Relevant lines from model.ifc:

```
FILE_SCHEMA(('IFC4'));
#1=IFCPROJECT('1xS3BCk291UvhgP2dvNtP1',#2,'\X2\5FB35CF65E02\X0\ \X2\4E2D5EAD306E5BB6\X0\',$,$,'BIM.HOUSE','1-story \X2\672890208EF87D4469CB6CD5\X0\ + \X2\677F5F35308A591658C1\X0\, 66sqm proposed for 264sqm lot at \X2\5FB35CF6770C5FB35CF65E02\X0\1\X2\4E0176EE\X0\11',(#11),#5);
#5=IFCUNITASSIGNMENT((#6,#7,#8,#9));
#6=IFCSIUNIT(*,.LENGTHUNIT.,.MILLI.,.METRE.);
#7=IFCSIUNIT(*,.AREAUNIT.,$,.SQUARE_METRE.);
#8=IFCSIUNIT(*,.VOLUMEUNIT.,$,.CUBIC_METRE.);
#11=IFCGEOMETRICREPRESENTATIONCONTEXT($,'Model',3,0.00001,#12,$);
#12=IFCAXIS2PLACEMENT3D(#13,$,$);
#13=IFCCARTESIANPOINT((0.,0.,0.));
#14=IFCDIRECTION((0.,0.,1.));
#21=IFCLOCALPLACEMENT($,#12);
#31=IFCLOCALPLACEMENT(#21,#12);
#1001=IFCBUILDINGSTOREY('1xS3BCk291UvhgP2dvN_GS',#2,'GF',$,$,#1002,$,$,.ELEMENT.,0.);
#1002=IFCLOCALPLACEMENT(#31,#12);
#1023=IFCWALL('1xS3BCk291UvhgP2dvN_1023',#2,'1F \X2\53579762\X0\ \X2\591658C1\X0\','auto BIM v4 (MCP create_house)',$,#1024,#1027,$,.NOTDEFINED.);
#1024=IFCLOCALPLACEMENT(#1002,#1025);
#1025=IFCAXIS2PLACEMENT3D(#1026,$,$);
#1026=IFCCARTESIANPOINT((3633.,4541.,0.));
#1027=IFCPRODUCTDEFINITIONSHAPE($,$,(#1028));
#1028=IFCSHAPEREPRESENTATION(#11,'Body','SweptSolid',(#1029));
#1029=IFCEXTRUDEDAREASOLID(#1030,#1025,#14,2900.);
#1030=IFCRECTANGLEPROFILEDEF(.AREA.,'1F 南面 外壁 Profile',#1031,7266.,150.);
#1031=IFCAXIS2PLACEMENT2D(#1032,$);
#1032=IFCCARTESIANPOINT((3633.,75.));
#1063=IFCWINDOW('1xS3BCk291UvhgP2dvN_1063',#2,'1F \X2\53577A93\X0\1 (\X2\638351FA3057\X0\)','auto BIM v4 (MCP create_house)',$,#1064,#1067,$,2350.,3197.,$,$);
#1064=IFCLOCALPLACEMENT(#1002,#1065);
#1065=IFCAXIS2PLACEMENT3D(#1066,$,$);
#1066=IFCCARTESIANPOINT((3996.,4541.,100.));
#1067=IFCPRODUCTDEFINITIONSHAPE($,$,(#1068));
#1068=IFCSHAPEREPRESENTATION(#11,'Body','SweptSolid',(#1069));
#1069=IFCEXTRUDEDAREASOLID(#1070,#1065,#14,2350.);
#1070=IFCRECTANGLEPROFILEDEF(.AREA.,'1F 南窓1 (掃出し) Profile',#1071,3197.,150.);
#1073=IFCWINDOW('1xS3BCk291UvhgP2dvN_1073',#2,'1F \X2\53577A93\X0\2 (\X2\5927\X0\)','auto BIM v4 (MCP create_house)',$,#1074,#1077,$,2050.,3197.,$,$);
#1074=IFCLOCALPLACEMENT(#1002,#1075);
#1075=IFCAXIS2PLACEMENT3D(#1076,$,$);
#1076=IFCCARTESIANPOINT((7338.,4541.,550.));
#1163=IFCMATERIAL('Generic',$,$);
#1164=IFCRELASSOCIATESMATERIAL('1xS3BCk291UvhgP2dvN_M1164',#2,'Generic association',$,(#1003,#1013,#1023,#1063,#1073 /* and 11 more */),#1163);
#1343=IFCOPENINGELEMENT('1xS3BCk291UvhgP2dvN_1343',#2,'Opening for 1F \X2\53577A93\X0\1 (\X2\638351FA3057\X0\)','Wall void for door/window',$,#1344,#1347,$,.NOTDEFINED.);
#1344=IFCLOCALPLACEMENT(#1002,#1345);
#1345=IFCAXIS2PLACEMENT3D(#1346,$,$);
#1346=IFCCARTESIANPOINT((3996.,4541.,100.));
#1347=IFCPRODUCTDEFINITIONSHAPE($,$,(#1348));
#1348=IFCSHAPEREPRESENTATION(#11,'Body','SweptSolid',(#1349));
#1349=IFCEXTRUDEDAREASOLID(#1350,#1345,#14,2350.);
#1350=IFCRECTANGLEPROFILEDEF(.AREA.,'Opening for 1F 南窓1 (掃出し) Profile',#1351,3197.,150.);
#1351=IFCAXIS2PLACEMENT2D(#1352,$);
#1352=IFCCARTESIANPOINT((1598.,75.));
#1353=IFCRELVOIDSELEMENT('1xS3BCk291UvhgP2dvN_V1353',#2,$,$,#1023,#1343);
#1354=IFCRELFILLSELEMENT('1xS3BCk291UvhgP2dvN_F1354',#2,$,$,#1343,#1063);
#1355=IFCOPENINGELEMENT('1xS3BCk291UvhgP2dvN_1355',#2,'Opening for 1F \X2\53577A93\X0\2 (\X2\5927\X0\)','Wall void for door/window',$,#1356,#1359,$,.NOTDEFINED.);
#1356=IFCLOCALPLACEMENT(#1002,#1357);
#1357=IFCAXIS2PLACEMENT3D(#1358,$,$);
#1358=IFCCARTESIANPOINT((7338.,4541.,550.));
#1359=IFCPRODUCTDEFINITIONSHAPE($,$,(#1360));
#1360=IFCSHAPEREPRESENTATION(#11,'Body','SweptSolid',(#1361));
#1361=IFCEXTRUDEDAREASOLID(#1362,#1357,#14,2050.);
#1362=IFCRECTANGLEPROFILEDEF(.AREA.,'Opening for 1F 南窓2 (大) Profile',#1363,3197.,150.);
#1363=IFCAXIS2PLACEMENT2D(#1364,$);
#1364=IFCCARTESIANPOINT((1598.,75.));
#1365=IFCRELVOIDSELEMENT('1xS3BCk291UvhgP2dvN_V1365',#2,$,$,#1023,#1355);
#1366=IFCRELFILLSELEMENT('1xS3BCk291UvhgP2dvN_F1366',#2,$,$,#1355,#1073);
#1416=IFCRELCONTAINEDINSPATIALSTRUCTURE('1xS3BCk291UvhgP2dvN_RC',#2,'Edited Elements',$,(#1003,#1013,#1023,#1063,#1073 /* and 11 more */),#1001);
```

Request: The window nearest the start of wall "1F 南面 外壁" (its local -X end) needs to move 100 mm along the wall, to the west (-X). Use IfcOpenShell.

```python
import ifcopenshell
import ifcopenshell.api.geometry
import ifcopenshell.util.placement

model = ifcopenshell.open("model.ifc")

window = model.by_guid("1xS3BCk291UvhgP2dvN_1063")
opening = window.FillsVoids[0].RelatingOpeningElement
wall = opening.VoidsElements[0].RelatingBuildingElement

wall_matrix = ifcopenshell.util.placement.get_local_placement(wall.ObjectPlacement)
shift = wall_matrix[:3, 0] * -100.0
before = ifcopenshell.util.placement.get_local_placement(window.ObjectPlacement)[:3, 3].copy()

# The window is not placed relative to its opening, so move both.
for product in (opening, window):
    matrix = ifcopenshell.util.placement.get_local_placement(product.ObjectPlacement)
    matrix[:3, 3] += shift
    ifcopenshell.api.geometry.edit_object_placement(model, product=product, matrix=matrix, is_si=False)

after = ifcopenshell.util.placement.get_local_placement(window.ObjectPlacement)[:3, 3]
print("window moved by", (after - before).round(3) + 0.0)

model.write("model_edited.ifc")
```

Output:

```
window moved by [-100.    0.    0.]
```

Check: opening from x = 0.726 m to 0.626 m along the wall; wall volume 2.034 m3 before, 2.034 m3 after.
